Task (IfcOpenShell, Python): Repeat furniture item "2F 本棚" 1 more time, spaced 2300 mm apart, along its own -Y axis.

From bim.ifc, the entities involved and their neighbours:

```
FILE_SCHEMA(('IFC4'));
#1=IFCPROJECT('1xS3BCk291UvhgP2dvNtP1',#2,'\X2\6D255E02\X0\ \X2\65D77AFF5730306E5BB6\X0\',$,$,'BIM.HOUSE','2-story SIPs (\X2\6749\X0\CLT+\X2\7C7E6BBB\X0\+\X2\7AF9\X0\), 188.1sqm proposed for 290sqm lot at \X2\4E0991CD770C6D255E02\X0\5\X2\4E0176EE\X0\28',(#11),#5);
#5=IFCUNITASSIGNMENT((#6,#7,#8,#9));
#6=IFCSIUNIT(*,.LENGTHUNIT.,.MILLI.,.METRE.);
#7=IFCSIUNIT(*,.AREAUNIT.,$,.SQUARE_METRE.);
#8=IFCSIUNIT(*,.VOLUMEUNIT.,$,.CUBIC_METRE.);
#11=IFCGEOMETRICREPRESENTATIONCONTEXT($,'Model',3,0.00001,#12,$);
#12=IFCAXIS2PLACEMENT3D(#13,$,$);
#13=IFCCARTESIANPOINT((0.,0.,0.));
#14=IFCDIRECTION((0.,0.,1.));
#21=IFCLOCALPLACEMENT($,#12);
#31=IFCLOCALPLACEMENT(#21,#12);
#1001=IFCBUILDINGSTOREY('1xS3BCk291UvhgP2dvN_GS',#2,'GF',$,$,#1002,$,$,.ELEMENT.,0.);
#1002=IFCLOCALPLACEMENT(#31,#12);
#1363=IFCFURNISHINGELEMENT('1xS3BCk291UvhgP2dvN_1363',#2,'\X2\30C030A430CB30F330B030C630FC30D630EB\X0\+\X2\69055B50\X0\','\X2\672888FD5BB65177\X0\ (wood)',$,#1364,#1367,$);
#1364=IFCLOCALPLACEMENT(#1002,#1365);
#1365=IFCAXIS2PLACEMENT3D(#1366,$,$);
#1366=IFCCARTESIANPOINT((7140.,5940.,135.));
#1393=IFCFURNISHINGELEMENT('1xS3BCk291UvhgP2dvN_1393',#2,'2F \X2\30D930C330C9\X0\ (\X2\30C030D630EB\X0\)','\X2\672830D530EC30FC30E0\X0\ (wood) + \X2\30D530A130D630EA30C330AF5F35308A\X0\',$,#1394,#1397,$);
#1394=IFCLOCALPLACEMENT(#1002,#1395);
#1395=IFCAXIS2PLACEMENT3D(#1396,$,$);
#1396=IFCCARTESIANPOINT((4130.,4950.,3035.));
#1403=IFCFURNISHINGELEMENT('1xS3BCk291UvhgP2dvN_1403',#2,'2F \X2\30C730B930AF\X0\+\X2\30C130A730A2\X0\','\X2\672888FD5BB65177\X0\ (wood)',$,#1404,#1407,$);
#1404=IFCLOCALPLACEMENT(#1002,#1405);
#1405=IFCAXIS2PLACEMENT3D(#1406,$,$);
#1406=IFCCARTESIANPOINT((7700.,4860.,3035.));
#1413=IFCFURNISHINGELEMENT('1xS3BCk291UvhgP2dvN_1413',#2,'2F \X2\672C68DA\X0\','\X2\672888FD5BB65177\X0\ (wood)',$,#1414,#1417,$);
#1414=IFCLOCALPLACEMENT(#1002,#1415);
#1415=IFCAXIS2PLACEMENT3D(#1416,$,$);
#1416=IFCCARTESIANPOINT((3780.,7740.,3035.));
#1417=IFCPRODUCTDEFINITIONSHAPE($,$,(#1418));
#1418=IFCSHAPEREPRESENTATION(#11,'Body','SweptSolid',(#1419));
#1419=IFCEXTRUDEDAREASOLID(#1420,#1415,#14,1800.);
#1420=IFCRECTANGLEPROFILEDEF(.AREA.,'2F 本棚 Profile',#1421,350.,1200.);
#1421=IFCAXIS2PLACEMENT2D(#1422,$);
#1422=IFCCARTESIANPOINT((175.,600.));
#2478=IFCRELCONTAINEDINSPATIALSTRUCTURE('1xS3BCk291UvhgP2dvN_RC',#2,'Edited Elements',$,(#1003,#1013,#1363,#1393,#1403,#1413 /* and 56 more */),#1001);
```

```python
import ifcopenshell
import ifcopenshell.api.geometry
import ifcopenshell.api.root
import ifcopenshell.util.element
import ifcopenshell.util.placement
import ifcopenshell.util.unit

model = ifcopenshell.open("bim.ifc")
unit_scale = ifcopenshell.util.unit.calculate_unit_scale(model)


def reuse_history(source, copy):
    """copy_class also copies each property set's owner history, people and application; keep the originals."""
    for rel in copy.IsDefinedBy:
        if rel.is_a("IfcRelDefinesByProperties") and (history := rel.RelatingPropertyDefinition.OwnerHistory):
            rel.RelatingPropertyDefinition.OwnerHistory = source.OwnerHistory
            ifcopenshell.util.element.remove_deep2(model, history)


source = model.by_id(1413)
base = ifcopenshell.util.placement.get_local_placement(source.ObjectPlacement)
step = -base[:3, 1] * 2.3 / unit_scale

for i in range(1, 2):
    copy = ifcopenshell.api.root.copy_class(model, product=source)
    copy.Representation = ifcopenshell.util.element.copy_deep(
        model, source.Representation, exclude=["IfcGeometricRepresentationContext", "IfcRepresentationMap"]
    )
    reuse_history(source, copy)
    matrix = base.copy()
    matrix[:3, 3] += i * step
    print("added at", matrix[:3, 3].round(3) + 0.0)
    ifcopenshell.api.geometry.edit_object_placement(model, product=copy, matrix=matrix, is_si=False)

model.write("bim_updated.ifc")
```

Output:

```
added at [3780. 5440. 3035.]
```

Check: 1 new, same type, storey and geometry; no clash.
